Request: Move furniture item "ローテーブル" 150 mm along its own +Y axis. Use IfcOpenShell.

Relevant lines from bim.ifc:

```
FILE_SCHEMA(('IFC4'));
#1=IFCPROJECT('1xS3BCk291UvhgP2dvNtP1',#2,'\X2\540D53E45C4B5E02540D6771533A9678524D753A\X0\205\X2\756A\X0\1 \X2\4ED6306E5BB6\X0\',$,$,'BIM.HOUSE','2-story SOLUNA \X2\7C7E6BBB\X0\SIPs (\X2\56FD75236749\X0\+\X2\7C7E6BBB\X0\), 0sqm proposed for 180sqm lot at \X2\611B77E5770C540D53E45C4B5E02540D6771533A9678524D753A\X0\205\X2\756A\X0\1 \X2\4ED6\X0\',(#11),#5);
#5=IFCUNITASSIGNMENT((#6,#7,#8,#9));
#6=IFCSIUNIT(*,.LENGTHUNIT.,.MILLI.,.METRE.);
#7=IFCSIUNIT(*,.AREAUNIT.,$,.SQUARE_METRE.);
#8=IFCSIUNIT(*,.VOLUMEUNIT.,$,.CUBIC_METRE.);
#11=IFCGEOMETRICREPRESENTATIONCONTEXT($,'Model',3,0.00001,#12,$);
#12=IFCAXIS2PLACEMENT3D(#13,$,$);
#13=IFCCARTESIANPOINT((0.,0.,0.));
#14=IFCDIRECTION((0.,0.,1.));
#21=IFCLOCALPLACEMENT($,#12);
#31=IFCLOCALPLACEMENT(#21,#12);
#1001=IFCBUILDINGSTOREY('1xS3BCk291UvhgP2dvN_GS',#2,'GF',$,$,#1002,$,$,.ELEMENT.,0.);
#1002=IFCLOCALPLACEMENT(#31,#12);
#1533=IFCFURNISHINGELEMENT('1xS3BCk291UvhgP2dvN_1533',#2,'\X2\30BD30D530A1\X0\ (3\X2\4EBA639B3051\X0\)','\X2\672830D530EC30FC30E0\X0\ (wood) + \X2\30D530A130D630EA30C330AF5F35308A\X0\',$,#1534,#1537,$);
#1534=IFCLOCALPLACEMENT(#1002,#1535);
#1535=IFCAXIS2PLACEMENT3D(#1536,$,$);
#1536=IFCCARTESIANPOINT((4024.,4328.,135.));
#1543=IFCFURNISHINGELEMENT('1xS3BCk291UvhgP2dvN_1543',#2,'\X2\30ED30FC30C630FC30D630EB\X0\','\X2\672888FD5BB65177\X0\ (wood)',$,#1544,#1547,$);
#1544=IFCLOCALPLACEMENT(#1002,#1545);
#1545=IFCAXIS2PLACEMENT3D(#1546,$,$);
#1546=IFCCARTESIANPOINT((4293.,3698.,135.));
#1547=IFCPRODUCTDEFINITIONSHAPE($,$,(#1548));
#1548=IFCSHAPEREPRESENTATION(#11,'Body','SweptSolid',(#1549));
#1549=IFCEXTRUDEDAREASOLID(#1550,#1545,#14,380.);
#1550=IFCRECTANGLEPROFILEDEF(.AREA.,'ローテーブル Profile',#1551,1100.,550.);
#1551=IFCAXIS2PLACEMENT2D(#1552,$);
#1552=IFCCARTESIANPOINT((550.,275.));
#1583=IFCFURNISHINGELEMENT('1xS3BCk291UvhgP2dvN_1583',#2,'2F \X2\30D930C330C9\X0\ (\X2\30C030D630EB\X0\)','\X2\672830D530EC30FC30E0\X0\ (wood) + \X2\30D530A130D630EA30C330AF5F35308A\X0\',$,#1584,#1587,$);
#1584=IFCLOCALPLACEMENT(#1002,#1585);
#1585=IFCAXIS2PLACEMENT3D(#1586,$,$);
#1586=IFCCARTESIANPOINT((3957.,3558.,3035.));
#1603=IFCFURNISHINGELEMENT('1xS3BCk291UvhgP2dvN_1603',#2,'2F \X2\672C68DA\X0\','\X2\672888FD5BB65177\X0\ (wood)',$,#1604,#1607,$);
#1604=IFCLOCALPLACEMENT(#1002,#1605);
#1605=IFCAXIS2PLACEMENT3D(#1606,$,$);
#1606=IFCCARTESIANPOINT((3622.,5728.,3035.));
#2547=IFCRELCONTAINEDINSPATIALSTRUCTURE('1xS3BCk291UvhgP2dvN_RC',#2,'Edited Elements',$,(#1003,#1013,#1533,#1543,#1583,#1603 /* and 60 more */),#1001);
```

```python
import ifcopenshell
import ifcopenshell.api.geometry
import ifcopenshell.util.placement
import ifcopenshell.util.unit

model = ifcopenshell.open("bim.ifc")
unit_scale = ifcopenshell.util.unit.calculate_unit_scale(model)

item = model.by_guid("1xS3BCk291UvhgP2dvN_1543")
matrix = ifcopenshell.util.placement.get_local_placement(item.ObjectPlacement)
matrix[:3, 3] += matrix[:3, 1] * 0.15 / unit_scale
ifcopenshell.api.geometry.edit_object_placement(model, product=item, matrix=matrix, is_si=False)

print(ifcopenshell.util.placement.get_local_placement(item.ObjectPlacement).round(3) + 0.0)

model.write("bim-out.ifc")
```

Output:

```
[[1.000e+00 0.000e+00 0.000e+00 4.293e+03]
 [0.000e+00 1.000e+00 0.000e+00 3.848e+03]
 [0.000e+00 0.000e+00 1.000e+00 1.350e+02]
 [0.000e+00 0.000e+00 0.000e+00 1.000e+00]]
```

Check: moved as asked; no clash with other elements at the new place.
